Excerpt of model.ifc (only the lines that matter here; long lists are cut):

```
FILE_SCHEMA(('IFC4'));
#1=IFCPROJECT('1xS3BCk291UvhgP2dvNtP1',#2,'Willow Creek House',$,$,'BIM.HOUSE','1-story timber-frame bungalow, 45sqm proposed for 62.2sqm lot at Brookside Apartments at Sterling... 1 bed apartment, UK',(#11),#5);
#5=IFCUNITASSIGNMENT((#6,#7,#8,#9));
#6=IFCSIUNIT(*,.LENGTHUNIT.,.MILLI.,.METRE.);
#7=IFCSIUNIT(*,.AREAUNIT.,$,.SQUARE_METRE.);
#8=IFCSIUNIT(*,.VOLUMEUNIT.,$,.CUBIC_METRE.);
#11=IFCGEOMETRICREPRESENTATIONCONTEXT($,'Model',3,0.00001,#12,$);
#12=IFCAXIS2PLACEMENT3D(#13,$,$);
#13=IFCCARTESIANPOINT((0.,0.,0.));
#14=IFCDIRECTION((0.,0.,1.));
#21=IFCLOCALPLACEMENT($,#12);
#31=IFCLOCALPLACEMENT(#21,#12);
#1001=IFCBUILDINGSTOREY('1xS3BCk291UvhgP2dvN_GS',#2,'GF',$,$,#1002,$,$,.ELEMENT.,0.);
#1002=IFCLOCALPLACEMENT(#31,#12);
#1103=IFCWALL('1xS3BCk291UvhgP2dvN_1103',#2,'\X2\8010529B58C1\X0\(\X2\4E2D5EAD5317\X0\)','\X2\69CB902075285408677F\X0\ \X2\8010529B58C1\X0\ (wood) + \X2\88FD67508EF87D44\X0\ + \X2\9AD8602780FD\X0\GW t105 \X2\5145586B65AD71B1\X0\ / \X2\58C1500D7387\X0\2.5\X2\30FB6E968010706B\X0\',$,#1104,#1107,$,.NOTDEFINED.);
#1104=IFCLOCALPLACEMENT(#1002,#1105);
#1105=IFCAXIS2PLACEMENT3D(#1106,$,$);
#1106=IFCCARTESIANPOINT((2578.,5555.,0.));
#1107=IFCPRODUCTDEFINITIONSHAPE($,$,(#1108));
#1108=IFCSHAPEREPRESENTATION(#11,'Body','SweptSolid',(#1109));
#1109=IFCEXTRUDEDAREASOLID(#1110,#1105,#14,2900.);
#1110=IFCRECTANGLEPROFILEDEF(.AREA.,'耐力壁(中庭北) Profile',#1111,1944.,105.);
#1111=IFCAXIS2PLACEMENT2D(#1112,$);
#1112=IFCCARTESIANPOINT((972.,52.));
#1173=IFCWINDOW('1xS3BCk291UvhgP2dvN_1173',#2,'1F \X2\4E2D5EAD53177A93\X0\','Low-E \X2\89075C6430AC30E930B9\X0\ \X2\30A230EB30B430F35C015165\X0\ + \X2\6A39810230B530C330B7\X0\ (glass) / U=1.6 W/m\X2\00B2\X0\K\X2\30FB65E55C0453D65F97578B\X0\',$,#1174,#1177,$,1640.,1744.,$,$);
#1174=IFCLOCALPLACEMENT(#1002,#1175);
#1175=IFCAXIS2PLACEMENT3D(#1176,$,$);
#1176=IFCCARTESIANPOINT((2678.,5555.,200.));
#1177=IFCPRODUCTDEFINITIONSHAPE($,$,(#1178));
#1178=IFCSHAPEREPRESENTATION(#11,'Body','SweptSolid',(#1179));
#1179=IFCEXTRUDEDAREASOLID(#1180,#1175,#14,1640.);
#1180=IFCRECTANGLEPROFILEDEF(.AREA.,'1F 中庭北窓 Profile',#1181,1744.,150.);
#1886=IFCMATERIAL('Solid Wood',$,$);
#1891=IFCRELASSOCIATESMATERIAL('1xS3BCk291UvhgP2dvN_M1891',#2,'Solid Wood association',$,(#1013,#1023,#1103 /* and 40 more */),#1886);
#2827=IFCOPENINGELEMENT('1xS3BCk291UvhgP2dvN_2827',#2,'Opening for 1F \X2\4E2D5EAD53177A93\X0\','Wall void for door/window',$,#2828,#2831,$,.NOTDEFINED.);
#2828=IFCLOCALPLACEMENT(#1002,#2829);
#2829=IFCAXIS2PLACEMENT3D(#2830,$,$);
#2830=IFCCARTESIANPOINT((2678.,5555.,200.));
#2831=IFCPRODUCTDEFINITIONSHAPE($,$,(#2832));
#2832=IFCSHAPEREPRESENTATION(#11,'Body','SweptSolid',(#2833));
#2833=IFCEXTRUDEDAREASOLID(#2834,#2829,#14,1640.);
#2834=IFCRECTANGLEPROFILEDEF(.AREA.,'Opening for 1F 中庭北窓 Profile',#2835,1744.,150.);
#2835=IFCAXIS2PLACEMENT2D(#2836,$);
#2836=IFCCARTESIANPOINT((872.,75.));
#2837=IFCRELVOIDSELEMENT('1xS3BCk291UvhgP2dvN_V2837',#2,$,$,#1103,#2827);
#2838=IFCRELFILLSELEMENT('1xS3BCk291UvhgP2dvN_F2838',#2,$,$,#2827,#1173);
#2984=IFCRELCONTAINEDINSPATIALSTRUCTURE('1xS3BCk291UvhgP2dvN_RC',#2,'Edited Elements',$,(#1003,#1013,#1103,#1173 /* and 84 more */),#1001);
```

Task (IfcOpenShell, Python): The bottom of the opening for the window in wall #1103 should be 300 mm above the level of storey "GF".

```python
import numpy as np
import ifcopenshell
import ifcopenshell.api.geometry
import ifcopenshell.geom
import ifcopenshell.util.element
import ifcopenshell.util.placement
import ifcopenshell.util.shape
import ifcopenshell.util.unit

model = ifcopenshell.open("model.ifc")
unit_scale = ifcopenshell.util.unit.calculate_unit_scale(model)

window = model.by_guid("1xS3BCk291UvhgP2dvN_1173")
opening = window.FillsVoids[0].RelatingOpeningElement
storey = ifcopenshell.util.element.get_container(window, ifc_class="IfcBuildingStorey")
level = ifcopenshell.util.placement.get_local_placement(storey.ObjectPlacement)[2, 3]

# The opening's origin need not be at the sill, so measure its lowest point.
shape = ifcopenshell.geom.create_shape(ifcopenshell.geom.settings(), opening)
bottom = ifcopenshell.util.shape.get_shape_bottom_elevation(shape, shape.geometry) / unit_scale
dz = level + 0.3 / unit_scale - bottom

shift = np.array([0.0, 0.0, dz])
# The window is not placed relative to its opening, so move both.
for product in (opening, window):
    matrix = ifcopenshell.util.placement.get_local_placement(product.ObjectPlacement)
    matrix[:3, 3] += shift
    ifcopenshell.api.geometry.edit_object_placement(model, product=product, matrix=matrix, is_si=False)

print(f"moved by {dz * unit_scale:+.3f} m")

model.write("model-out.ifc")
```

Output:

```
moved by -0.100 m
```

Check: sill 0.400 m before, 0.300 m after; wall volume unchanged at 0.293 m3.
